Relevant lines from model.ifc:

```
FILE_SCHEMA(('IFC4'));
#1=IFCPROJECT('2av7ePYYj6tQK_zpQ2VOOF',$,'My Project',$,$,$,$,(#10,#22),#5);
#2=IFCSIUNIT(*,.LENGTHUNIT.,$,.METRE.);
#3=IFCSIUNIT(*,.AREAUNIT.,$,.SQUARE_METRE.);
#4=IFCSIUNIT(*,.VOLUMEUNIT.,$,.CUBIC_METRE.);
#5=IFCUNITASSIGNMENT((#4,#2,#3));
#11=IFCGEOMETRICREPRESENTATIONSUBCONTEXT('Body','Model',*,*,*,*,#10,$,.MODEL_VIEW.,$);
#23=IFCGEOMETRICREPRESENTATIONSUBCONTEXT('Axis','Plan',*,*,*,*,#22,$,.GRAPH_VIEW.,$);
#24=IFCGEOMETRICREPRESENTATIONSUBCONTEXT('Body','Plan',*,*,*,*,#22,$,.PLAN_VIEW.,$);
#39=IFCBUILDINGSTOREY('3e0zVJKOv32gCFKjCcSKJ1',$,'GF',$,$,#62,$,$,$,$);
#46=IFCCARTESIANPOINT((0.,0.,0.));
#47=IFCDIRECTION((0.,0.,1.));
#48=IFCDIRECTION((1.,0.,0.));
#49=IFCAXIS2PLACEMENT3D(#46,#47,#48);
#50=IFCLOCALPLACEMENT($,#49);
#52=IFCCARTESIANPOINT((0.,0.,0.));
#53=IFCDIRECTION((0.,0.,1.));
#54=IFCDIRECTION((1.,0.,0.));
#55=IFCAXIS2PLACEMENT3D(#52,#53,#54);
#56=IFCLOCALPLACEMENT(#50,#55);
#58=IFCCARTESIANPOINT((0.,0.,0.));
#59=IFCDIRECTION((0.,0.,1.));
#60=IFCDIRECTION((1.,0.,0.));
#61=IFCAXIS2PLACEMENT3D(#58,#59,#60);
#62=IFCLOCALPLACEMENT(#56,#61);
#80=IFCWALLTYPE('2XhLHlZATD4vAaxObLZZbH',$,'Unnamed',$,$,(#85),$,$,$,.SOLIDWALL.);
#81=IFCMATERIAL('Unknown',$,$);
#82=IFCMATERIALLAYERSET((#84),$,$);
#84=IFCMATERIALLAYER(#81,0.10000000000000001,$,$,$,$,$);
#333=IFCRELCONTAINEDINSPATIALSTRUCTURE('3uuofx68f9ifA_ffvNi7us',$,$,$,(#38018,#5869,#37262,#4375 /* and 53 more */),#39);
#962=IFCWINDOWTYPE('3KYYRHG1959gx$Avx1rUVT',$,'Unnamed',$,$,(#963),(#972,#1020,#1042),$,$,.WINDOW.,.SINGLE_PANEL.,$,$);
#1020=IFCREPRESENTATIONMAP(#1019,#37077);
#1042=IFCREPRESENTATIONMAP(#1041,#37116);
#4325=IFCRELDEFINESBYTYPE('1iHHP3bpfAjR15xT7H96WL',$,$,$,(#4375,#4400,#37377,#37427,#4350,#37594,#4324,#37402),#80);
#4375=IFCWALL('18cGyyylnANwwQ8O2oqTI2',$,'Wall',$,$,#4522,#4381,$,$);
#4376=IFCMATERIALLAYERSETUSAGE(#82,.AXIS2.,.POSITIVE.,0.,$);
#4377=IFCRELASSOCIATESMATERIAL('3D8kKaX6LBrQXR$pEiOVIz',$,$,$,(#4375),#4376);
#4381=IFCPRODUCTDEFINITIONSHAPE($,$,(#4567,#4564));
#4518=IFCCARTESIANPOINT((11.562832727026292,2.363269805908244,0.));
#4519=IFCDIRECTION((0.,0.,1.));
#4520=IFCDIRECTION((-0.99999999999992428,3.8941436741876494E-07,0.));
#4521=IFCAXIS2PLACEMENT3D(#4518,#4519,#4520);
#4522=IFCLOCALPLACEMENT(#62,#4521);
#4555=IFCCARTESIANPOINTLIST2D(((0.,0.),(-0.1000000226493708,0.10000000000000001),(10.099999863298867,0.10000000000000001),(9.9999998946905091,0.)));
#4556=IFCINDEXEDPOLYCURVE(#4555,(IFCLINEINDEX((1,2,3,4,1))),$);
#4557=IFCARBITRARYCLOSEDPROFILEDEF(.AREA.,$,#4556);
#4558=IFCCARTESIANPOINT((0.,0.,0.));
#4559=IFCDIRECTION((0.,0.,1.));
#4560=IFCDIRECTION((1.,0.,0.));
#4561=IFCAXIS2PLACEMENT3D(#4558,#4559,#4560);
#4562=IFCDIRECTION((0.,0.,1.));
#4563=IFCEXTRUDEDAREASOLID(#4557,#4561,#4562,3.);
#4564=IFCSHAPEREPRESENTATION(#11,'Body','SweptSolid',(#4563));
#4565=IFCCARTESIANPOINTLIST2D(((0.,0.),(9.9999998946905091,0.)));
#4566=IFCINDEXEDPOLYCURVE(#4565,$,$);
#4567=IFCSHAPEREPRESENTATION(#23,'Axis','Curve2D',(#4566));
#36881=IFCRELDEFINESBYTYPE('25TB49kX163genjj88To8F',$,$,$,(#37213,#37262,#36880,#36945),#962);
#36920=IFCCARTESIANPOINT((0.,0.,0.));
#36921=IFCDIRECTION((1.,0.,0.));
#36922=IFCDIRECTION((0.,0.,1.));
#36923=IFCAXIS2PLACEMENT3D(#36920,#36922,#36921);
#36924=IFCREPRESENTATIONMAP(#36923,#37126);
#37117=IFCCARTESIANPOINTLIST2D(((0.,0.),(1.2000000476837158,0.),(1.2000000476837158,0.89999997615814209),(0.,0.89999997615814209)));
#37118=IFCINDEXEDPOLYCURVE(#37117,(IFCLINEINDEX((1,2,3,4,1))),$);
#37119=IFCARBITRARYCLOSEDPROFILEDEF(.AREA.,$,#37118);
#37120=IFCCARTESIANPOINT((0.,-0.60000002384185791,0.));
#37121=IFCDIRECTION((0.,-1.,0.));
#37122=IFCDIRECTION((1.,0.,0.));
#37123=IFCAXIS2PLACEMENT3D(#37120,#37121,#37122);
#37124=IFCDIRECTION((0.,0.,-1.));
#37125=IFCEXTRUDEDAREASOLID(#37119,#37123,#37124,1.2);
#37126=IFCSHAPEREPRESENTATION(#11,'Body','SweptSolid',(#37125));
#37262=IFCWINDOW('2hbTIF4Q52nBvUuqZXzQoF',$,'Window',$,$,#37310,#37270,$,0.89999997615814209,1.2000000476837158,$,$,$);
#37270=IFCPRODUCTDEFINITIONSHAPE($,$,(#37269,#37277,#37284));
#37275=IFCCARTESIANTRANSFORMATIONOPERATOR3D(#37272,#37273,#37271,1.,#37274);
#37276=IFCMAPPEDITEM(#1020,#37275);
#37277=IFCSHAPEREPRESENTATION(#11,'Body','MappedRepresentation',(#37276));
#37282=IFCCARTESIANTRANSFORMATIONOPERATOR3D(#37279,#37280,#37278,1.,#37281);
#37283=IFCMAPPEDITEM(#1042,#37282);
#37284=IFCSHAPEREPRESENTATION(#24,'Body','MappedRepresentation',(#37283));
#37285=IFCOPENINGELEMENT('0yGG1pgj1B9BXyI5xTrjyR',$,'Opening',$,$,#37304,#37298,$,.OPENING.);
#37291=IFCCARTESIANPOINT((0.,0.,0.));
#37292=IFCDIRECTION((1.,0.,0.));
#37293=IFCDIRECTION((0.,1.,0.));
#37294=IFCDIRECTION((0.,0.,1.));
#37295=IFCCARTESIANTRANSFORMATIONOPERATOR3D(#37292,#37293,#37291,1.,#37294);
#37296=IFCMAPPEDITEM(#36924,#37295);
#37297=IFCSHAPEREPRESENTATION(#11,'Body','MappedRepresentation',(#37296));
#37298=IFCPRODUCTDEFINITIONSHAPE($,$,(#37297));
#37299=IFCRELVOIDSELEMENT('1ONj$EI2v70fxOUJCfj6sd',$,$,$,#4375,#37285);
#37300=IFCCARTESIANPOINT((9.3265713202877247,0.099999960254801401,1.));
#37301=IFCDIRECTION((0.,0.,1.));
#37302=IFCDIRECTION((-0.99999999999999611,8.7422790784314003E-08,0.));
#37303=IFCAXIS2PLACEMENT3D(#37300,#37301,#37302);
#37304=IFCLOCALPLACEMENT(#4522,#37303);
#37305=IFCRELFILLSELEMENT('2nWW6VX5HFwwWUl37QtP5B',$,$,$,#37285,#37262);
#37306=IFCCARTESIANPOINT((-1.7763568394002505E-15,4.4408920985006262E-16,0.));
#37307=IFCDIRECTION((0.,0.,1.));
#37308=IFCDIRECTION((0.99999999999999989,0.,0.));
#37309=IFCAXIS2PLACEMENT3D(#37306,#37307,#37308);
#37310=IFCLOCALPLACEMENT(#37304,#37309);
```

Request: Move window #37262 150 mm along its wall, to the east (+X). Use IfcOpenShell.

```python
import ifcopenshell
import ifcopenshell.api.geometry
import ifcopenshell.util.placement
import ifcopenshell.util.unit

model = ifcopenshell.open("model.ifc")
unit_scale = ifcopenshell.util.unit.calculate_unit_scale(model)

window = model.by_id(37262)
opening = window.FillsVoids[0].RelatingOpeningElement
wall = opening.VoidsElements[0].RelatingBuildingElement

wall_matrix = ifcopenshell.util.placement.get_local_placement(wall.ObjectPlacement)
shift = wall_matrix[:3, 0] * -0.15 / unit_scale
before = ifcopenshell.util.placement.get_local_placement(window.ObjectPlacement)[:3, 3].copy()

# The window is placed relative to its opening, so it follows when the opening moves.
matrix = ifcopenshell.util.placement.get_local_placement(opening.ObjectPlacement)
matrix[:3, 3] += shift
ifcopenshell.api.geometry.edit_object_placement(
    model, product=opening, matrix=matrix, is_si=False, should_transform_children=True
)

after = ifcopenshell.util.placement.get_local_placement(window.ObjectPlacement)[:3, 3]
print("window moved by", (after - before).round(3) + 0.0)

model.write("model_updated.ifc")
```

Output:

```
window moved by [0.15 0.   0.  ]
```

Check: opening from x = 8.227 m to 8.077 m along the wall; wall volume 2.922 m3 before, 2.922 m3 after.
